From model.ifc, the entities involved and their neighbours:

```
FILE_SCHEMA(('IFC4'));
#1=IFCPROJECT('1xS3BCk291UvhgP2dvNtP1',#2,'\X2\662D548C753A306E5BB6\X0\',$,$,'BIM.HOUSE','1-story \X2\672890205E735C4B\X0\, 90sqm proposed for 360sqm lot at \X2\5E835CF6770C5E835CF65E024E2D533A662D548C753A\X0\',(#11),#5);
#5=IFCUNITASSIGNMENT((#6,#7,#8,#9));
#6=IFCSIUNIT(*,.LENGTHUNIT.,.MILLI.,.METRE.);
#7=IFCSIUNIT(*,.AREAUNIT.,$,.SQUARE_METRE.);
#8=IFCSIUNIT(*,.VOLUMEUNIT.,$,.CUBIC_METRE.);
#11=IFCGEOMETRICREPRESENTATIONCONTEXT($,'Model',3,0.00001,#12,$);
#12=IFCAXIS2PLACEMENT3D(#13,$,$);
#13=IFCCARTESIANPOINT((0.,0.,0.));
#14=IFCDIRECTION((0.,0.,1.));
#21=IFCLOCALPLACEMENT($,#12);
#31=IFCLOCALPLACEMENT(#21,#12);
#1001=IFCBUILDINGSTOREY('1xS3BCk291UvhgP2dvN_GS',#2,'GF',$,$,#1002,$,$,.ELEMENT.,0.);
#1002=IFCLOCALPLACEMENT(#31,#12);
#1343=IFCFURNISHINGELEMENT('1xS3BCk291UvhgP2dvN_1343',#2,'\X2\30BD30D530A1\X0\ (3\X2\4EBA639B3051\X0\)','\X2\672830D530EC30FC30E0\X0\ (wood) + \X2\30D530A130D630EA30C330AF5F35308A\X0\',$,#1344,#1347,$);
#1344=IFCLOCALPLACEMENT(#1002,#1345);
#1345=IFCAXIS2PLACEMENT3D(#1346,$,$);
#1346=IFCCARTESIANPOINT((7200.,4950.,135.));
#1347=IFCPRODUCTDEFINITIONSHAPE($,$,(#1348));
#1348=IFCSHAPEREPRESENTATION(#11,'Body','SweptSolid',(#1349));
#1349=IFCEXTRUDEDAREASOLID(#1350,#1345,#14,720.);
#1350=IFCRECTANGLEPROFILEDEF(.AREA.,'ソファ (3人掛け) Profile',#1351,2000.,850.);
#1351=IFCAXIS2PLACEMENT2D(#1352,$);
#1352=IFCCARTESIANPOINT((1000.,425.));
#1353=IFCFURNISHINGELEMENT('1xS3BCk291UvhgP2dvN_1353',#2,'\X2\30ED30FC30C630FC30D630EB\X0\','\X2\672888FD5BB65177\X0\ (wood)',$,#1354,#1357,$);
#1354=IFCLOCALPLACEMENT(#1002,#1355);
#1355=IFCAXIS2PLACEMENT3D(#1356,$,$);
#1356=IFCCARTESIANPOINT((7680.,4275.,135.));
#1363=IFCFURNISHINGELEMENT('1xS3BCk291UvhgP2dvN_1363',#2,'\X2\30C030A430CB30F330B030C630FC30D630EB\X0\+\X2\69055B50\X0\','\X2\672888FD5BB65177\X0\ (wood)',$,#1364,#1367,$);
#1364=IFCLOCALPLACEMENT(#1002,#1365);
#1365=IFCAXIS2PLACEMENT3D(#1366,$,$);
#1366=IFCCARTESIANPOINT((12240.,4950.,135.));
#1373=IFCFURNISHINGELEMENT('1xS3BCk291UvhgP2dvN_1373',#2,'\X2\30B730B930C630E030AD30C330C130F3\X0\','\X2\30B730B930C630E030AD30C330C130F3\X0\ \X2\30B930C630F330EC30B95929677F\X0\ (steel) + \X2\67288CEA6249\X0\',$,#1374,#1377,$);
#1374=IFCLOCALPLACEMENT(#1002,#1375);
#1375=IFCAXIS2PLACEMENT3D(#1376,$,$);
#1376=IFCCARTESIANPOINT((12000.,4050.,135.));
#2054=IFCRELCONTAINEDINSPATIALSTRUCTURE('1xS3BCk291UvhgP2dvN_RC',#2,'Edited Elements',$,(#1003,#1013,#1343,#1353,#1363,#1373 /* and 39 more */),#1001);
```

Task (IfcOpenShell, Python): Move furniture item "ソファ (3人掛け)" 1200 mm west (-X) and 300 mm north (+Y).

```python
import ifcopenshell
import ifcopenshell.api.geometry
import ifcopenshell.util.placement

model = ifcopenshell.open("model.ifc")

item = model.by_guid("1xS3BCk291UvhgP2dvN_1343")
matrix = ifcopenshell.util.placement.get_local_placement(item.ObjectPlacement)
matrix[0, 3] -= 1200.0
matrix[1, 3] += 300.0
ifcopenshell.api.geometry.edit_object_placement(model, product=item, matrix=matrix, is_si=False)

print(ifcopenshell.util.placement.get_local_placement(item.ObjectPlacement).round(3) + 0.0)

model.write("model_updated.ifc")
```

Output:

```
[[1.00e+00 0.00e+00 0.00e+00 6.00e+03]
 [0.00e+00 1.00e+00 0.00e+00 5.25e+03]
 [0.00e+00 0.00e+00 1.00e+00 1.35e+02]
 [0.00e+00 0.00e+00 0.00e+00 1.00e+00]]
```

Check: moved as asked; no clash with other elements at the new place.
